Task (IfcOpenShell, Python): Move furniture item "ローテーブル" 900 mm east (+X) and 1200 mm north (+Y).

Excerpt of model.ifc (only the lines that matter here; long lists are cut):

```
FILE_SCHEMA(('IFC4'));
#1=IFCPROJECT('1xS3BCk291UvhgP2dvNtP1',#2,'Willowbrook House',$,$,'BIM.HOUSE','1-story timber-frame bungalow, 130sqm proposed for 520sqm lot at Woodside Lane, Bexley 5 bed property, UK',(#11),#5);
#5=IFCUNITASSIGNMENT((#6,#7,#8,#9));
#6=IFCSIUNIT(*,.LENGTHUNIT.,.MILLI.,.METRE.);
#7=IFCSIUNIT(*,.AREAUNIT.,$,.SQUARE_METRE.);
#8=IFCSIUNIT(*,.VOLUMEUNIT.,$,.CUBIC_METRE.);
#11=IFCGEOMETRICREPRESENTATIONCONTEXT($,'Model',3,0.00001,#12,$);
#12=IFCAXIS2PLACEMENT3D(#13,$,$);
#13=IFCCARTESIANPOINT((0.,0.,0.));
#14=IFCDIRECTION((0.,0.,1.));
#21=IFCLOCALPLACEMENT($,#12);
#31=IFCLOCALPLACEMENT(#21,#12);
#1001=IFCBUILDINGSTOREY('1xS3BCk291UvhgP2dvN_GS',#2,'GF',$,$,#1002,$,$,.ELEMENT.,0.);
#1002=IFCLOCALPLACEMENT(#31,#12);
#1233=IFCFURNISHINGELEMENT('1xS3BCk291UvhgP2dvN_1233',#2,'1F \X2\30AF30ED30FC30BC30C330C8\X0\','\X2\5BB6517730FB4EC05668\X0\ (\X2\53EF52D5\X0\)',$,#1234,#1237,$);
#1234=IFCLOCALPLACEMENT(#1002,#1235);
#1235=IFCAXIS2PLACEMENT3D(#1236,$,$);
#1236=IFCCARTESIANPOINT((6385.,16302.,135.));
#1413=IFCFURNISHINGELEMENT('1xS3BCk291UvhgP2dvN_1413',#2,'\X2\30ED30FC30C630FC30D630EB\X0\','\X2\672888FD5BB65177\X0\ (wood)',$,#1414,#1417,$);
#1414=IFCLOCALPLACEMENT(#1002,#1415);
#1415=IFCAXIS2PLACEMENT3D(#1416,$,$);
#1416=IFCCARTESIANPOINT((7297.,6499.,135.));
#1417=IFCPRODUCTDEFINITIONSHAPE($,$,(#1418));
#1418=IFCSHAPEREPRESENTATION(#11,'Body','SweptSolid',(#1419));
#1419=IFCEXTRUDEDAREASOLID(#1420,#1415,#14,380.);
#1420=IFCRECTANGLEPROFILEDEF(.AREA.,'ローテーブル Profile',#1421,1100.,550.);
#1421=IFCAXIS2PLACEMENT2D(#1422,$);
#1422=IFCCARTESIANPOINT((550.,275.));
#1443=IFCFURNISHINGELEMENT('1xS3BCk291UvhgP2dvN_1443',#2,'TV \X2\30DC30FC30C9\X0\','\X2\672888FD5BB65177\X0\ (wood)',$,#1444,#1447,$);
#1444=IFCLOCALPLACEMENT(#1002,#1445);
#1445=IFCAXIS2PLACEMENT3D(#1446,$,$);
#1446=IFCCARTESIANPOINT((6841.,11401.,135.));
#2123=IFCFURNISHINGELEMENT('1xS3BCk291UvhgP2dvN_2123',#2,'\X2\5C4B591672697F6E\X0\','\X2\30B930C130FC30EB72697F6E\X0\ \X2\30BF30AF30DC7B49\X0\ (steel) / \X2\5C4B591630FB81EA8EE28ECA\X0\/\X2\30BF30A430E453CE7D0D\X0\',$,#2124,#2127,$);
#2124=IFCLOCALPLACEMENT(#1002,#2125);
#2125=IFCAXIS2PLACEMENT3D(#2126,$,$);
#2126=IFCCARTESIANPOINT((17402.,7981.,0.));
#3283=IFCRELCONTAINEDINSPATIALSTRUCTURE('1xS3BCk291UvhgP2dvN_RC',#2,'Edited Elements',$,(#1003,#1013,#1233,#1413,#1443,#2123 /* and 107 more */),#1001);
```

```python
import ifcopenshell
import ifcopenshell.api.geometry
import ifcopenshell.util.placement

model = ifcopenshell.open("model.ifc")

item = model.by_id(1413)
matrix = ifcopenshell.util.placement.get_local_placement(item.ObjectPlacement)
matrix[0, 3] += 900.0
matrix[1, 3] += 1200.0
ifcopenshell.api.geometry.edit_object_placement(model, product=item, matrix=matrix, is_si=False)

print(ifcopenshell.util.placement.get_local_placement(item.ObjectPlacement).round(3) + 0.0)

model.write("model_v2.ifc")
```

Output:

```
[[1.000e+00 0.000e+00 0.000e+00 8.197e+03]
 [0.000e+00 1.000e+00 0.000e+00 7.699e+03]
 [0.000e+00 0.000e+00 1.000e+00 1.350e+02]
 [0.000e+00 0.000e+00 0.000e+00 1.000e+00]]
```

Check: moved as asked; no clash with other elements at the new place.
